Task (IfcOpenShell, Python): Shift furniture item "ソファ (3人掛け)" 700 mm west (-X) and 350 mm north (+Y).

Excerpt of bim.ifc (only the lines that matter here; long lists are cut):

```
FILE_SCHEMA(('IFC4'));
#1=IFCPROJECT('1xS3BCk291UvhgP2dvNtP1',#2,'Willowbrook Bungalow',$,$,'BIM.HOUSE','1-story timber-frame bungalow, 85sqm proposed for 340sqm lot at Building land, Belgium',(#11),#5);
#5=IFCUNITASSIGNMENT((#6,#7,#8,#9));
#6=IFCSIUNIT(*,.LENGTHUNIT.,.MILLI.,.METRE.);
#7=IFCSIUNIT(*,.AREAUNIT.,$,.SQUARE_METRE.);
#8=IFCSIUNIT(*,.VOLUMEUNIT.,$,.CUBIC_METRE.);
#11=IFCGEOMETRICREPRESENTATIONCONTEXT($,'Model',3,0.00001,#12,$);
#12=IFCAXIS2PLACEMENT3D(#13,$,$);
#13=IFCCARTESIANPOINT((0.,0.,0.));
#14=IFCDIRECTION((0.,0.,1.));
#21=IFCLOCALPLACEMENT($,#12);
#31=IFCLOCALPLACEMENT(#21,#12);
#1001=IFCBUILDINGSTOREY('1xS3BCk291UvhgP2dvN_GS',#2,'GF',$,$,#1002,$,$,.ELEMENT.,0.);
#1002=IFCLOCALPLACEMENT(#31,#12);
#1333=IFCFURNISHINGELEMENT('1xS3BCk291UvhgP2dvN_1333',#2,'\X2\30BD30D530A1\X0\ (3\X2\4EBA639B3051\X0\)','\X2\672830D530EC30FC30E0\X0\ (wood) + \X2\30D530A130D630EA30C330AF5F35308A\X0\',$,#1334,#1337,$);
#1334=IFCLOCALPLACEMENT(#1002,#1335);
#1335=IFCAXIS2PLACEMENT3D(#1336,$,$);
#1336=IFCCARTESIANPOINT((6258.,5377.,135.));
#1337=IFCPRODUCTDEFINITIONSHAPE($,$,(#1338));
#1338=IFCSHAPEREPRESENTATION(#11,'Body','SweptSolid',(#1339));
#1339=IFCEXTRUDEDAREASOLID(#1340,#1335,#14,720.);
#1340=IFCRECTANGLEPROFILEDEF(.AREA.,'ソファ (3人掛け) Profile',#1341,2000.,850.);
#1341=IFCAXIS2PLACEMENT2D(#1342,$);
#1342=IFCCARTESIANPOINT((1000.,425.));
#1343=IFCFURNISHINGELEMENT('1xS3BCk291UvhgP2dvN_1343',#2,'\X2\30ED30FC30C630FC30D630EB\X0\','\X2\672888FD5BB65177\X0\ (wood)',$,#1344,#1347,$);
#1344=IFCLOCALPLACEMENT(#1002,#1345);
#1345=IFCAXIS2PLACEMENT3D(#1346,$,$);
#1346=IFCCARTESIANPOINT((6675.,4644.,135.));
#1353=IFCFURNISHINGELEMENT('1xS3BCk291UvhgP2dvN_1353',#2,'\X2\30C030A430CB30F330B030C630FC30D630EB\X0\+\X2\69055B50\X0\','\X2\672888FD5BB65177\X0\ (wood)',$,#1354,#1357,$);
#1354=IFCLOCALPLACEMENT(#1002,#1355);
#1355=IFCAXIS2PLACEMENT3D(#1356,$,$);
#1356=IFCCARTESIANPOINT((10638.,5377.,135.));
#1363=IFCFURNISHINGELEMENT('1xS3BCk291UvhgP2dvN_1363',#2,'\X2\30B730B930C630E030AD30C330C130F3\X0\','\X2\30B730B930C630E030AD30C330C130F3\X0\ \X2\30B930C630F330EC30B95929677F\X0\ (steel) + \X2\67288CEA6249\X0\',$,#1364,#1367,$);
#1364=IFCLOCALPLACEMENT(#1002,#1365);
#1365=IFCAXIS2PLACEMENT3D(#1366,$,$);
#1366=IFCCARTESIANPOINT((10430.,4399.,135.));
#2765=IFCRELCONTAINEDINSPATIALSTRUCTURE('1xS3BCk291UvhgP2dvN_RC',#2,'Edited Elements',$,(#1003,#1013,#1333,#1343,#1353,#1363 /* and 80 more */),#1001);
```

```python
import ifcopenshell
import ifcopenshell.api.geometry
import ifcopenshell.util.placement

model = ifcopenshell.open("bim.ifc")

item = model.by_id(1333)
matrix = ifcopenshell.util.placement.get_local_placement(item.ObjectPlacement)
matrix[0, 3] -= 700.0
matrix[1, 3] += 350.0
ifcopenshell.api.geometry.edit_object_placement(model, product=item, matrix=matrix, is_si=False)

print(ifcopenshell.util.placement.get_local_placement(item.ObjectPlacement).round(3) + 0.0)

model.write("bim_edited.ifc")
```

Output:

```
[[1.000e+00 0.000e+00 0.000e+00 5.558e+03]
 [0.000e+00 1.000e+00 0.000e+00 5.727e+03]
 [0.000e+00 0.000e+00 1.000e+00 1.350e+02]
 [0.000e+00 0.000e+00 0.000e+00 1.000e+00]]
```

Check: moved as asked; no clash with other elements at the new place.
